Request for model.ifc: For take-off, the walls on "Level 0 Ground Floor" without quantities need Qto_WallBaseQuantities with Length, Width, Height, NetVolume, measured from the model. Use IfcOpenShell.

First a look at what the model holds.

```python
import ifcopenshell
import ifcopenshell.util.element
import ifcopenshell.util.unit

model = ifcopenshell.open("model.ifc")
print(model.schema)
for unit_type in ("LENGTHUNIT", "AREAUNIT", "VOLUMEUNIT"):
    print(unit_type, ifcopenshell.util.unit.calculate_unit_scale(model, unit_type))
storey = next(s for s in model.by_type("IfcBuildingStorey") if s.Name == "Level 0 Ground Floor")
walls = [e for e in ifcopenshell.util.element.get_decomposition(storey) if e.is_a("IfcWall")]
for e in sorted(walls, key=lambda e: e.id()):
    print(e.id(), e.is_a(), e.Name, list(ifcopenshell.util.element.get_psets(e, qtos_only=True)), sep=" | ")
```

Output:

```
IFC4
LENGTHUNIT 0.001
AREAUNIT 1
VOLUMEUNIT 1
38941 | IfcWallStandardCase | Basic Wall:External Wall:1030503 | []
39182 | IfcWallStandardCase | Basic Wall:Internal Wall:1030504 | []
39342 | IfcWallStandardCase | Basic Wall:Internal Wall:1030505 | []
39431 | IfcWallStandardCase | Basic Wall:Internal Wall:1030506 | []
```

```python
import ifcopenshell
import ifcopenshell.api.pset
import ifcopenshell.geom
import ifcopenshell.util.element
import ifcopenshell.util.shape
import ifcopenshell.util.unit

model = ifcopenshell.open("model.ifc")
unit_scale = ifcopenshell.util.unit.calculate_unit_scale(model)
volume_scale = ifcopenshell.util.unit.calculate_unit_scale(model, "VOLUMEUNIT")
settings = ifcopenshell.geom.settings()

storey = next(s for s in model.by_type("IfcBuildingStorey") if s.Name == "Level 0 Ground Floor")
walls = [e for e in ifcopenshell.util.element.get_decomposition(storey) if e.is_a("IfcWall")]

for e in sorted(walls, key=lambda e: e.id()):
    if ifcopenshell.util.element.get_psets(e, qtos_only=True, should_inherit=False):
        continue
    # Geometry comes back in metres, in the element's own axes.
    shape = ifcopenshell.geom.create_shape(settings, e)
    values = {
        "Length": ifcopenshell.util.shape.get_x(shape.geometry) / unit_scale,
        "Width": ifcopenshell.util.shape.get_y(shape.geometry) / unit_scale,
        "Height": ifcopenshell.util.shape.get_z(shape.geometry) / unit_scale,
        "NetVolume": ifcopenshell.util.shape.get_volume(shape.geometry) / volume_scale,
    }
    qto = ifcopenshell.api.pset.add_qto(model, product=e, name="Qto_WallBaseQuantities")
    ifcopenshell.api.pset.edit_qto(model, qto=qto, properties=values)
    print(e.id(), {k: round(v, 3) for k, v in values.items()})

model.write("model_edited.ifc")
```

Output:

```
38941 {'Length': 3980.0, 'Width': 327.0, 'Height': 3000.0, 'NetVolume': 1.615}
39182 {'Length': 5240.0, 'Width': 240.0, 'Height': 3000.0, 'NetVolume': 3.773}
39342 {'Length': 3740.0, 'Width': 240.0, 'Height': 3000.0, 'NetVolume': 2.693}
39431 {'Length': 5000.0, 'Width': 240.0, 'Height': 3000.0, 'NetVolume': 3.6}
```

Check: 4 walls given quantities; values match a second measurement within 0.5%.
